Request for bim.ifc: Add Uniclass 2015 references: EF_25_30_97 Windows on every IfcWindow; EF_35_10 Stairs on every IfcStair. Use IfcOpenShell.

First a look at what the model holds.

```python
import ifcopenshell

model = ifcopenshell.open("bim.ifc")
print(model.schema)
print("classifications:", [c.Name for c in model.by_type("IfcClassification")])
for ifc_class in ("IfcDoor", "IfcRoof", "IfcStair", "IfcWall", "IfcWindow"):
    print(ifc_class, len(model.by_type(ifc_class)))
```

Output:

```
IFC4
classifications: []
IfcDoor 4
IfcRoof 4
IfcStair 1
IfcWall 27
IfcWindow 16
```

```python
import ifcopenshell
import ifcopenshell.api.classification

model = ifcopenshell.open("bim.ifc")

system = ifcopenshell.api.classification.add_classification(model, classification="Uniclass 2015")

codes = {
    "IfcWindow": ("EF_25_30_97", "Windows"),
    "IfcStair": ("EF_35_10", "Stairs"),
}
for ifc_class, (code, name) in codes.items():
    products = model.by_type(ifc_class)
    ifcopenshell.api.classification.add_reference(
        model, products=products, classification=system, identification=code, name=name
    )
    print(code, len(products))

model.write("bim_updated.ifc")
```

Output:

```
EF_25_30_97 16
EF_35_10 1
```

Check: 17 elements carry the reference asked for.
